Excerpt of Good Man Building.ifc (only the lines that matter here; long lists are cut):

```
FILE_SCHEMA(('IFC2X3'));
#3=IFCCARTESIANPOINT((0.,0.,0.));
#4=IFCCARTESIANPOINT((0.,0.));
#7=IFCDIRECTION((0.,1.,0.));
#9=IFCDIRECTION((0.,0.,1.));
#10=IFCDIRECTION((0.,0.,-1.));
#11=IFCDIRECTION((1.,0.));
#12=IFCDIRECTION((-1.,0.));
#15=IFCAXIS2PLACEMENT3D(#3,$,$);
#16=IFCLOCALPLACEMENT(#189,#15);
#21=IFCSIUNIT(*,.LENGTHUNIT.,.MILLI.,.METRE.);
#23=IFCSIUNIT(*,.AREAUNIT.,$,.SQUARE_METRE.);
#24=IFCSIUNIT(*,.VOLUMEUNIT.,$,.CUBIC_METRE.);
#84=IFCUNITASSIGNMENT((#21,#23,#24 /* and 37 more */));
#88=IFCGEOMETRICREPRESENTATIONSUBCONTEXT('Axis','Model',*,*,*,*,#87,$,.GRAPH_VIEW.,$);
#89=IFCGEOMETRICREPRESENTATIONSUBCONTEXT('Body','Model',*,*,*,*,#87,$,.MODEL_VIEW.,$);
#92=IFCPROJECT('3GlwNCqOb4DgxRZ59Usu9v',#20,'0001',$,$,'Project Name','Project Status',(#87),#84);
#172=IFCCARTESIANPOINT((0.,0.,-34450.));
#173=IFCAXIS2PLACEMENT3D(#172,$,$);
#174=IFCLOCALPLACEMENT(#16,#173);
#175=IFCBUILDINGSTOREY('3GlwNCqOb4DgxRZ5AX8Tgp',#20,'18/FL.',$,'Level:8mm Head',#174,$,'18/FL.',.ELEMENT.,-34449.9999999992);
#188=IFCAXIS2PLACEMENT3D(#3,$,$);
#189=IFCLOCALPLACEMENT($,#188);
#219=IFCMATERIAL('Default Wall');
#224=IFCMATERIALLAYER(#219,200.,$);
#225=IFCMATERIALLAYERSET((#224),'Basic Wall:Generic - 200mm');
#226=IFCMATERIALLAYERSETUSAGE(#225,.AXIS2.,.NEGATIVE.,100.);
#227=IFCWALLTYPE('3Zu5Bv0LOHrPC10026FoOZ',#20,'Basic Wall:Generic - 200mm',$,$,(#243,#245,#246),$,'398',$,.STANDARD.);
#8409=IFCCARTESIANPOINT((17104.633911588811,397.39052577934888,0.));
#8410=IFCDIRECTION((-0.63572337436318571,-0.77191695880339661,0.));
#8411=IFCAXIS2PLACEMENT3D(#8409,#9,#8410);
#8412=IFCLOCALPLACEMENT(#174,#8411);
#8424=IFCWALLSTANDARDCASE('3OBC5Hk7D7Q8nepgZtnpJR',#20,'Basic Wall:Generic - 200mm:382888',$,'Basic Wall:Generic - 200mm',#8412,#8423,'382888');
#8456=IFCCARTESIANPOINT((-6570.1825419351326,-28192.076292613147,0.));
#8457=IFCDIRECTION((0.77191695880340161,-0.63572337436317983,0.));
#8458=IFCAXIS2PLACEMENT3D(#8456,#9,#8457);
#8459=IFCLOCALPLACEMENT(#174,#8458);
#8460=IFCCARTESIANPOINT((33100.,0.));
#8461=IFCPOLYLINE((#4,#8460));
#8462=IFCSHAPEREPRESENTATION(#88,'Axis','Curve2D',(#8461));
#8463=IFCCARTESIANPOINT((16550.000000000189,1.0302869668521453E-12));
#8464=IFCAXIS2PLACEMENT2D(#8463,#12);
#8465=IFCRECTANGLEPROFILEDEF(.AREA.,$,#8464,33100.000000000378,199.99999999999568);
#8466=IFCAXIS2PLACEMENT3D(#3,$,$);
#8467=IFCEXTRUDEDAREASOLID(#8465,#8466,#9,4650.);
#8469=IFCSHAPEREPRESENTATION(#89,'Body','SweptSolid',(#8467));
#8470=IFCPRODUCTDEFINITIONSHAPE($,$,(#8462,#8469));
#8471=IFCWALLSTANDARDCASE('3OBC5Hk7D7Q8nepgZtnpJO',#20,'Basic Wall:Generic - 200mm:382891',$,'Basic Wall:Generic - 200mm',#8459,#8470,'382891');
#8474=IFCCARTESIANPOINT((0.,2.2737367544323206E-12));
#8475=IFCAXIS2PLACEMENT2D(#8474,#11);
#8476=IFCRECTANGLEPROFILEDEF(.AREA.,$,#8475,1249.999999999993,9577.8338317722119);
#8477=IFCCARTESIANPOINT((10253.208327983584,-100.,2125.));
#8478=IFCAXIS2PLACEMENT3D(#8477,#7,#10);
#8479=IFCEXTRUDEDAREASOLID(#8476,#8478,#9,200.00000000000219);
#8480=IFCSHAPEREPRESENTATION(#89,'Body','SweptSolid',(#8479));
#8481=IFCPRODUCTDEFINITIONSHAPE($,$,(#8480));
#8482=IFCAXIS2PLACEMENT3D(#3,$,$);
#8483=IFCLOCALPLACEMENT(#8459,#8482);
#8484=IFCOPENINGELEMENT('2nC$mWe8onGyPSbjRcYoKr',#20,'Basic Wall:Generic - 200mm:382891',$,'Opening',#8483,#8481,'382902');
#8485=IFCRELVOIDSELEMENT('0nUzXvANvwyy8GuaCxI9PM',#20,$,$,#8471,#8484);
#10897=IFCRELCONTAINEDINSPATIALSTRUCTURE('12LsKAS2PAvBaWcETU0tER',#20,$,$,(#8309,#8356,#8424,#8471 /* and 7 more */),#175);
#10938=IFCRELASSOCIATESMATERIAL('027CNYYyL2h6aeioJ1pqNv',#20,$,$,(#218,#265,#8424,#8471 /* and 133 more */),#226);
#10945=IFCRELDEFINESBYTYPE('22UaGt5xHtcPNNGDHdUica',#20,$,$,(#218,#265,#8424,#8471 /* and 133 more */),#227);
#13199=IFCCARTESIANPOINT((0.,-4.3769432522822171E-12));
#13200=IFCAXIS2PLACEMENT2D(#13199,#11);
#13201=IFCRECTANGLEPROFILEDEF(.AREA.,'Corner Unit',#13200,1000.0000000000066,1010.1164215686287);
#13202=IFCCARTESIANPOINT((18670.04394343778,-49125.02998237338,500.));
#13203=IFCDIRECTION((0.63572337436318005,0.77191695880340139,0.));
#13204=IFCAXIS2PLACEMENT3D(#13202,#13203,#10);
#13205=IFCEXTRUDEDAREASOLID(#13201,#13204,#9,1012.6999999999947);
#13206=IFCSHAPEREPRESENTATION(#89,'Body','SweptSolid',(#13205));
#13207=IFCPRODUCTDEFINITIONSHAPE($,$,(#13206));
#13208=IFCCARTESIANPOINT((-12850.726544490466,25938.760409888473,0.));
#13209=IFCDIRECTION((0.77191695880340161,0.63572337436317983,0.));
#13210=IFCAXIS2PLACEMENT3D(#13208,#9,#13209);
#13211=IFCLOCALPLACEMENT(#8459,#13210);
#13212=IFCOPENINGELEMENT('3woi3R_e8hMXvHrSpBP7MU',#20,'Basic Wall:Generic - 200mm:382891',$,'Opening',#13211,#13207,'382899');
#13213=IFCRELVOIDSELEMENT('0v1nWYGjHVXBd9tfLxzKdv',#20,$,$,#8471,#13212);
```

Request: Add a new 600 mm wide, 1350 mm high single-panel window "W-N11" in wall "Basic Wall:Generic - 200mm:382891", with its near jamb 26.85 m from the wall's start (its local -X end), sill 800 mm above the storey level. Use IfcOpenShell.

```python
import numpy as np
import ifcopenshell
import ifcopenshell.api.feature
import ifcopenshell.api.geometry
import ifcopenshell.api.root
import ifcopenshell.api.spatial
import ifcopenshell.api.type
import ifcopenshell.geom
import ifcopenshell.util.element
import ifcopenshell.util.placement
import ifcopenshell.util.representation
import ifcopenshell.util.shape
import ifcopenshell.util.unit

model = ifcopenshell.open("Good Man Building.ifc")
unit_scale = ifcopenshell.util.unit.calculate_unit_scale(model)
settings = ifcopenshell.geom.settings()


def volume(element):
    """Net volume in cubic metres, openings subtracted."""
    shape = ifcopenshell.geom.create_shape(settings, element)
    return ifcopenshell.util.shape.get_volume(shape.geometry)


wall = model.by_id(8471)
storey = ifcopenshell.util.element.get_container(wall, ifc_class="IfcBuildingStorey")
context = ifcopenshell.util.representation.get_context(model, "Model", "Body", "MODEL_VIEW")
before = volume(wall)

width, height, from_end, sill = 0.6, 1.35, 26.85, 0.8  # metres

# The wall runs along its own X axis, and the end named is its -X end.
wall_shape = ifcopenshell.geom.create_shape(settings, wall)
x, y, z = ifcopenshell.util.shape.get_vertices(wall_shape.geometry).T
start = x.min() + from_end
face, thickness = float(y.min()), float(y.max() - y.min())
wall_matrix = ifcopenshell.util.placement.get_local_placement(wall.ObjectPlacement)
level = ifcopenshell.util.placement.get_local_placement(storey.ObjectPlacement)[2, 3]


def in_wall(x, y):
    """Placement at x, y metres in the wall's axes, at sill height."""
    matrix = wall_matrix.copy()
    matrix[:, 3] = wall_matrix @ np.array([x / unit_scale, y / unit_scale, 0.0, 1.0])
    matrix[2, 3] = level + sill / unit_scale
    return matrix


# Opening: a box that overshoots both wall faces by 50 mm.
opening = ifcopenshell.api.root.create_entity(model, ifc_class="IfcOpeningElement")
box = ifcopenshell.api.geometry.add_wall_representation(
    model, context=context, length=width, height=height, thickness=thickness + 0.1
)
ifcopenshell.api.geometry.assign_representation(model, product=opening, representation=box)
ifcopenshell.api.geometry.edit_object_placement(model, product=opening, matrix=in_wall(start, face - 0.05), is_si=False)
ifcopenshell.api.feature.add_feature(model, feature=opening, element=wall)

window = ifcopenshell.api.root.create_entity(model, ifc_class="IfcWindow", name="W-N11")
window.OverallWidth, window.OverallHeight = width / unit_scale, height / unit_scale
body = ifcopenshell.api.geometry.add_window_representation(
    model,
    context=context,
    overall_width=window.OverallWidth,
    overall_height=window.OverallHeight,
    partition_type="SINGLE_PANEL",
)
ifcopenshell.api.geometry.assign_representation(model, product=window, representation=body)
ifcopenshell.api.spatial.assign_container(model, products=[window], relating_structure=storey)
fills = ifcopenshell.api.feature.add_filling(model, opening=opening, element=window)
fills.OwnerHistory = window.OwnerHistory  # required in IFC2X3

# IFC2X3 keeps the operation on the window style.
style = ifcopenshell.api.root.create_entity(model, ifc_class="IfcWindowStyle", name="W-N11")
style.OperationType, style.ConstructionType = "SINGLE_PANEL", "NOTDEFINED"
style.ParameterTakesPrecedence = style.Sizeable = False
ifcopenshell.api.type.assign_type(model, related_objects=[window], relating_type=style)

# Centre the window in the wall's thickness.
ifcopenshell.api.geometry.edit_object_placement(model, product=window, matrix=in_wall(start, face), is_si=False)
window_shape = ifcopenshell.geom.create_shape(settings, window)
depth = ifcopenshell.util.shape.get_vertices(window_shape.geometry)[:, 1]
offset = face + thickness / 2 - (depth.min() + depth.max()) / 2
ifcopenshell.api.geometry.edit_object_placement(model, product=window, matrix=in_wall(start, offset), is_si=False)

after = volume(wall)

print(f"wall volume {before:.3f} -> {after:.3f} m3")

model.write("Good Man Building_edited.ifc")
```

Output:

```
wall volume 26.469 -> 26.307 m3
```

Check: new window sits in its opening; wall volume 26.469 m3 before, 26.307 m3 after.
